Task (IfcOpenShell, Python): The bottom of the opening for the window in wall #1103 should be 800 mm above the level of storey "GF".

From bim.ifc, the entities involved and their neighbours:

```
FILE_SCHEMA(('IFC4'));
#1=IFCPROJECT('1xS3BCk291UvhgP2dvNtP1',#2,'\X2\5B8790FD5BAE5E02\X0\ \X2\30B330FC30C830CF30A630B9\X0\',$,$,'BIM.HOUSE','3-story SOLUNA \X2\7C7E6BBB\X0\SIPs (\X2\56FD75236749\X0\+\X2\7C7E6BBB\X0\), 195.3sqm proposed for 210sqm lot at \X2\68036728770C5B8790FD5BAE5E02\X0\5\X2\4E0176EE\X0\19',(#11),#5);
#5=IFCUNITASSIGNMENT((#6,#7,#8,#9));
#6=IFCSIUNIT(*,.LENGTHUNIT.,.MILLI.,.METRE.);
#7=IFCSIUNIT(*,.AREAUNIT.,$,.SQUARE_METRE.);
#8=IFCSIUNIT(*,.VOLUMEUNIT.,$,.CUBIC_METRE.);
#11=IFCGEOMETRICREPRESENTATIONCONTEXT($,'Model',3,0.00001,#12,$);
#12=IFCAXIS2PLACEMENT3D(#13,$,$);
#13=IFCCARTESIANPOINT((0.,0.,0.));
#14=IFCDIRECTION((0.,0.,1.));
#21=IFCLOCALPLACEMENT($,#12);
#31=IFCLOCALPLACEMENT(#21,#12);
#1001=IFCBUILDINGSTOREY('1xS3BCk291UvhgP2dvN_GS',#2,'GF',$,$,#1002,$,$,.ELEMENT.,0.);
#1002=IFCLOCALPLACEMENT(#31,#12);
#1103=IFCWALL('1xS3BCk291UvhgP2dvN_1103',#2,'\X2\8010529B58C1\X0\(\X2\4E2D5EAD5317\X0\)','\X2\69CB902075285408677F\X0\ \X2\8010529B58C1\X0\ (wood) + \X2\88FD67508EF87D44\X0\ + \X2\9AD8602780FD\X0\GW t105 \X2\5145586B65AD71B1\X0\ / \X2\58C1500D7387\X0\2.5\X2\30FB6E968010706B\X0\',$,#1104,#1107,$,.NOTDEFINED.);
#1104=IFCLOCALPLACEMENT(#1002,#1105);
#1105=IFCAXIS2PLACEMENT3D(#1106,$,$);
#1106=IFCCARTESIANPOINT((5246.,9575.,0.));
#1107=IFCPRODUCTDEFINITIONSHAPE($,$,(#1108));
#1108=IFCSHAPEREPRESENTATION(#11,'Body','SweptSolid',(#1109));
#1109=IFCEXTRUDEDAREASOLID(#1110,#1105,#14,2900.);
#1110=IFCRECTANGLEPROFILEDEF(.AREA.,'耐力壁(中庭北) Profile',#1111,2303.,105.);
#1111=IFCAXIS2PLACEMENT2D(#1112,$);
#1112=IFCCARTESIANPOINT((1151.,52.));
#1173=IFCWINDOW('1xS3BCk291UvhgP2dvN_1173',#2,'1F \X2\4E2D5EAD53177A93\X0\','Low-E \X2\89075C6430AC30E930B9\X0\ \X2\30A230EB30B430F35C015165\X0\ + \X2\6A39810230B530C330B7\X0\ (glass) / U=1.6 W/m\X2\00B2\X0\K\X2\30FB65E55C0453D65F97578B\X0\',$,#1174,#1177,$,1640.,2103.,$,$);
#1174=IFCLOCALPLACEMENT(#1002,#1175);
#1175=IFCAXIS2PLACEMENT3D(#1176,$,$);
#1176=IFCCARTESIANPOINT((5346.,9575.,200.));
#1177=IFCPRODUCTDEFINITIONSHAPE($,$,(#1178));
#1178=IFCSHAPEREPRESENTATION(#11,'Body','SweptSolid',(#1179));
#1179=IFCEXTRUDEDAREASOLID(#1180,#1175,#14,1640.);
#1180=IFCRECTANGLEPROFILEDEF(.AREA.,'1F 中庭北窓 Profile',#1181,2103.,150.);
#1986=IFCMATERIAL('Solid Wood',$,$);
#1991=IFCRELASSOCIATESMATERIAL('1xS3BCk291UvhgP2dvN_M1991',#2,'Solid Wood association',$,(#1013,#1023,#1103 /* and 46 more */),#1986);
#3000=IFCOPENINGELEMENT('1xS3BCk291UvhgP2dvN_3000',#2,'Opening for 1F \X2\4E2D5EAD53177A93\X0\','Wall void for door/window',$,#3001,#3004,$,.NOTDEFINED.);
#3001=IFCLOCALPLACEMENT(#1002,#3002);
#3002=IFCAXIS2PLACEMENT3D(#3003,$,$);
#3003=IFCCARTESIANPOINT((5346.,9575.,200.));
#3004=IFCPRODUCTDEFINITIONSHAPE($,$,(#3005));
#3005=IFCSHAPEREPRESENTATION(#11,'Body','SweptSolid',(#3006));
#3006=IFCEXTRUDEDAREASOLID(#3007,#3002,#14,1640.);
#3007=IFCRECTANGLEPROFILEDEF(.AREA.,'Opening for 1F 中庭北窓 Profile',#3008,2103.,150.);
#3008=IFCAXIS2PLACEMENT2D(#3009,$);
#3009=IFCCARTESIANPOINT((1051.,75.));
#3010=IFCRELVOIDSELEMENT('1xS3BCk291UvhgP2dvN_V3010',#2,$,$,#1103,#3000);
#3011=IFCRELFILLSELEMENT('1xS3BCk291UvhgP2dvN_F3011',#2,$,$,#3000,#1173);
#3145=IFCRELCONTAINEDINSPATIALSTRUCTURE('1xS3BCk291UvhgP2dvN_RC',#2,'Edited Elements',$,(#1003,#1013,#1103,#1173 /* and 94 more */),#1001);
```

```python
import numpy as np
import ifcopenshell
import ifcopenshell.api.geometry
import ifcopenshell.geom
import ifcopenshell.util.element
import ifcopenshell.util.placement
import ifcopenshell.util.shape
import ifcopenshell.util.unit

model = ifcopenshell.open("bim.ifc")
unit_scale = ifcopenshell.util.unit.calculate_unit_scale(model)

window = model.by_guid("1xS3BCk291UvhgP2dvN_1173")
opening = window.FillsVoids[0].RelatingOpeningElement
storey = ifcopenshell.util.element.get_container(window, ifc_class="IfcBuildingStorey")
level = ifcopenshell.util.placement.get_local_placement(storey.ObjectPlacement)[2, 3]

# The opening's origin need not be at the sill, so measure its lowest point.
shape = ifcopenshell.geom.create_shape(ifcopenshell.geom.settings(), opening)
bottom = ifcopenshell.util.shape.get_shape_bottom_elevation(shape, shape.geometry) / unit_scale
dz = level + 0.8 / unit_scale - bottom

shift = np.array([0.0, 0.0, dz])
# The window is not placed relative to its opening, so move both.
for product in (opening, window):
    matrix = ifcopenshell.util.placement.get_local_placement(product.ObjectPlacement)
    matrix[:3, 3] += shift
    ifcopenshell.api.geometry.edit_object_placement(model, product=product, matrix=matrix, is_si=False)

print(f"moved by {dz * unit_scale:+.3f} m")

model.write("bim_updated.ifc")
```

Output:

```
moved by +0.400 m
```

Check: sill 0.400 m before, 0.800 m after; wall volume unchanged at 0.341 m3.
